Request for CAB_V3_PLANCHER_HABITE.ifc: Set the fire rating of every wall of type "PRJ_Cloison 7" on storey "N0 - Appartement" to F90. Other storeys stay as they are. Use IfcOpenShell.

First a look at what the model holds.

```python
import ifcopenshell
import ifcopenshell.util.element

model = ifcopenshell.open("CAB_V3_PLANCHER_HABITE.ifc")
print(model.schema)
storey = next(s for s in model.by_type("IfcBuildingStorey") if s.Name == "N0 - Appartement")
walls = [e for e in ifcopenshell.util.element.get_decomposition(storey) if e.is_a("IfcWall")]
seen = {}
for e in walls:
    element_type = ifcopenshell.util.element.get_type(e)
    key = (element_type.Name if element_type != e and element_type else None, ifcopenshell.util.element.get_pset(e, "Pset_WallCommon", "FireRating"))
    seen[key] = seen.get(key, 0) + 1
for (name, value), count in sorted(seen.items(), key=str):
    print(count, "x", name, "|", value)
```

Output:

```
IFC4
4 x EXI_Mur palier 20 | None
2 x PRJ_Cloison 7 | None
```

```python
import ifcopenshell
import ifcopenshell.api.pset
import ifcopenshell.util.element

model = ifcopenshell.open("CAB_V3_PLANCHER_HABITE.ifc")

storey = next(s for s in model.by_type("IfcBuildingStorey") if s.Name == "N0 - Appartement")
walls = [e for e in ifcopenshell.util.element.get_decomposition(storey) if e.is_a("IfcWall")]

count = 0
for e in walls:
    element_type = ifcopenshell.util.element.get_type(e)
    if element_type in (None, e) or element_type.Name != "PRJ_Cloison 7":
        continue
    # add_pset returns the element's existing set when there is one.
    pset = ifcopenshell.api.pset.add_pset(model, product=e, name="Pset_WallCommon")
    ifcopenshell.api.pset.edit_pset(model, pset=pset, properties={"FireRating": "F90"})
    count += 1

print(count, "walls updated")

model.write("CAB_V3_PLANCHER_HABITE_updated.ifc")
```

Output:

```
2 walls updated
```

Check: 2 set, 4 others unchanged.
